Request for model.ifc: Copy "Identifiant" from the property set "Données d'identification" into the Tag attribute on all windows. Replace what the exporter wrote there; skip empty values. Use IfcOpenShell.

First a look at what the model holds.

```python
import ifcopenshell
import ifcopenshell.util.element

model = ifcopenshell.open("model.ifc")
print(model.schema)
windows = model.by_type("IfcWindow")
print(len(windows), "windows")
for e in windows[:8]:
    source = ifcopenshell.util.element.get_pset(e, "Données d'identification", "Identifiant")
    target = e.Tag
    print(e.id(), repr(source), repr(target), sep=" | ")
```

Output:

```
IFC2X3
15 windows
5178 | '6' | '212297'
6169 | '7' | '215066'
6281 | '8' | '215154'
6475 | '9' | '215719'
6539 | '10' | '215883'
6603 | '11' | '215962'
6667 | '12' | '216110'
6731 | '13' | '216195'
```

```python
import ifcopenshell
import ifcopenshell.util.element

model = ifcopenshell.open("model.ifc")

count = 0
for e in model.by_type("IfcWindow"):
    value = ifcopenshell.util.element.get_pset(e, "Données d'identification", "Identifiant")
    current = e.Tag
    if not value or not value.strip() or current == value:
        continue
    e.Tag = value
    count += 1

print(count, "windows updated")

model.write("model_rev.ifc")
```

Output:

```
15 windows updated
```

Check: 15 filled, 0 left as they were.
